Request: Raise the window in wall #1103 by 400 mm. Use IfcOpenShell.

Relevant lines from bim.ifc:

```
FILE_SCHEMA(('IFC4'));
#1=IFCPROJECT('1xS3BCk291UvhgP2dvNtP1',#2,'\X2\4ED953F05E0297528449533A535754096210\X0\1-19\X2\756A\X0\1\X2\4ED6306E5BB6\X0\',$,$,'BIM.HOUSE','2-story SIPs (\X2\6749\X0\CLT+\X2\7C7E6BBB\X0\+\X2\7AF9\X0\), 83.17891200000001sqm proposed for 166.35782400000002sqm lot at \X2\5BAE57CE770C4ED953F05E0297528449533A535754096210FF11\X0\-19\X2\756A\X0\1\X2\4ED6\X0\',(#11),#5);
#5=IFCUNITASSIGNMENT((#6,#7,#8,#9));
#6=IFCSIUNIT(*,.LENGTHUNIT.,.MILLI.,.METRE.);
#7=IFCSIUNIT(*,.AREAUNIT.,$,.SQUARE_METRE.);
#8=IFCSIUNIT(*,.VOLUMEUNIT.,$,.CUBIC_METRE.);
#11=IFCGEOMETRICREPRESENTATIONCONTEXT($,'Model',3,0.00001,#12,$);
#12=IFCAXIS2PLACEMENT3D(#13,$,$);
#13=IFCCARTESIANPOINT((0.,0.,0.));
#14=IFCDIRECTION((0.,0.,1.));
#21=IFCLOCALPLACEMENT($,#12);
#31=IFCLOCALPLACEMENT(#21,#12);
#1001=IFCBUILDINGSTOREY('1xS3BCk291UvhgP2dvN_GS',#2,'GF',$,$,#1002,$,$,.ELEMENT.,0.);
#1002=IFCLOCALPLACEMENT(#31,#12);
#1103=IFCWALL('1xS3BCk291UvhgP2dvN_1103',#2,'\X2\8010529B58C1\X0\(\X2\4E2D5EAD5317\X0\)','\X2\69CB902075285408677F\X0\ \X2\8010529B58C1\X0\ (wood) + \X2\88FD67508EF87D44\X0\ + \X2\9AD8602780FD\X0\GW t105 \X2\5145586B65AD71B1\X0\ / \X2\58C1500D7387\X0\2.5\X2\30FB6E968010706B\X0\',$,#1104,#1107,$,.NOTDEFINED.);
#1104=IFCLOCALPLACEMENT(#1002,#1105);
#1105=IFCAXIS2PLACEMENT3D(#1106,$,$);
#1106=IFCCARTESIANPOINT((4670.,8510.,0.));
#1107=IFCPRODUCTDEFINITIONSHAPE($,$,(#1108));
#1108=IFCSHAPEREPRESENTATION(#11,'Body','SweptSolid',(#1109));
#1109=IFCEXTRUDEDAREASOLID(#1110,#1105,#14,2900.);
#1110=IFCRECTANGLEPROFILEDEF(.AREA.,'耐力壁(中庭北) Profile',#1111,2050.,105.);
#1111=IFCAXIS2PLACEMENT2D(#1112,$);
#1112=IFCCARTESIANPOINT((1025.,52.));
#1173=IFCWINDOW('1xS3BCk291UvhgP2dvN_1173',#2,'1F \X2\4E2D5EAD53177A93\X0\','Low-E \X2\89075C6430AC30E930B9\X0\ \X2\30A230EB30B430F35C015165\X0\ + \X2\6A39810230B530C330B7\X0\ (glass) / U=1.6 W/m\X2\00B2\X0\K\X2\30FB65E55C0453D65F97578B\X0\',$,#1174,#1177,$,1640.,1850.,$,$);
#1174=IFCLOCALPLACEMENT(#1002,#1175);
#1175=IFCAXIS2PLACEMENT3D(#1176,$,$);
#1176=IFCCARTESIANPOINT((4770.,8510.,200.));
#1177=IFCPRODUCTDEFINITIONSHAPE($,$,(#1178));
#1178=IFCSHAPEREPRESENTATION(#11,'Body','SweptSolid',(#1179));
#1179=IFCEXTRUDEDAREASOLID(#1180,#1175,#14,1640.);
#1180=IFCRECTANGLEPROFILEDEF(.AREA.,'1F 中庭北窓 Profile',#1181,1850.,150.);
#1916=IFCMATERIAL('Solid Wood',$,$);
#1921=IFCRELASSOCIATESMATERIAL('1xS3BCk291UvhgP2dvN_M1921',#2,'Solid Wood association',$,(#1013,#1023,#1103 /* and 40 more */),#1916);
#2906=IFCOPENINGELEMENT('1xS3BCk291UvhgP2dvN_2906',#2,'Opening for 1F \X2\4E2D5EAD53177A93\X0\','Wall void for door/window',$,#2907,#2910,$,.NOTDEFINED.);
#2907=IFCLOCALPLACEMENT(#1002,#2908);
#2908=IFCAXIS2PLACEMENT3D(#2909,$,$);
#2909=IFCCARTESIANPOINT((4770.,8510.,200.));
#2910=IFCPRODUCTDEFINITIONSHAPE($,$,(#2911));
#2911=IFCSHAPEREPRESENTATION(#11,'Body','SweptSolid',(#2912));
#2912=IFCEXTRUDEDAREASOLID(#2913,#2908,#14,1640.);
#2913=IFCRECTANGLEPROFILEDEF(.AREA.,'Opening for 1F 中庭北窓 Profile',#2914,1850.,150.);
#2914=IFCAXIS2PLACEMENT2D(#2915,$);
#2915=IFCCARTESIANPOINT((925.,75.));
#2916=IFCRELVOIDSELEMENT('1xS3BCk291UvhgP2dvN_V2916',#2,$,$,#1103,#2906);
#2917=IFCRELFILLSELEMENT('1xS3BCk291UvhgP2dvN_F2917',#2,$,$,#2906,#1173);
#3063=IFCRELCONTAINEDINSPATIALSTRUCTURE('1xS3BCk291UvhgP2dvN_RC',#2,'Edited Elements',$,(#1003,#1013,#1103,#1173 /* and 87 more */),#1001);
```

```python
import numpy as np
import ifcopenshell
import ifcopenshell.api.geometry
import ifcopenshell.util.placement
import ifcopenshell.util.unit

model = ifcopenshell.open("bim.ifc")
unit_scale = ifcopenshell.util.unit.calculate_unit_scale(model)

window = model.by_guid("1xS3BCk291UvhgP2dvN_1173")
opening = window.FillsVoids[0].RelatingOpeningElement
dz = 400.0

shift = np.array([0.0, 0.0, dz])
# The window is not placed relative to its opening, so move both.
for product in (opening, window):
    matrix = ifcopenshell.util.placement.get_local_placement(product.ObjectPlacement)
    matrix[:3, 3] += shift
    ifcopenshell.api.geometry.edit_object_placement(model, product=product, matrix=matrix, is_si=False)

print(f"moved by {dz * unit_scale:+.3f} m")

model.write("bim-out.ifc")
```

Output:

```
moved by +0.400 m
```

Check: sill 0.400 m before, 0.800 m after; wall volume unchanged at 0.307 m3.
